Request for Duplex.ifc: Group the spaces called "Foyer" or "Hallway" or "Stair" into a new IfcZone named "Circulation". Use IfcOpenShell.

First a look at what the model holds.

```python
import ifcopenshell

model = ifcopenshell.open("Duplex.ifc")
print(model.schema)
seen = {}
for space in model.by_type("IfcSpace"):
    seen[space.LongName] = seen.get(space.LongName, 0) + 1
for name, count in sorted(seen.items(), key=str):
    print(count, "x", name)
print("zones:", [z.Name for z in model.by_type("IfcZone")][:20])
```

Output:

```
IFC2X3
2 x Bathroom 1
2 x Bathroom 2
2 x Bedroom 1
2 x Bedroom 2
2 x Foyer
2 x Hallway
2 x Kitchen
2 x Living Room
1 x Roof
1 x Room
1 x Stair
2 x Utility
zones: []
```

```python
import ifcopenshell
import ifcopenshell.api.group
import ifcopenshell.api.root

model = ifcopenshell.open("Duplex.ifc")

names = {"Foyer", "Hallway", "Stair"}
spaces = [s for s in model.by_type("IfcSpace") if s.LongName in names]

zone = ifcopenshell.api.root.create_entity(model, ifc_class="IfcZone", name="Circulation")
ifcopenshell.api.group.assign_group(model, products=spaces, group=zone)
print(len(spaces), "spaces in", zone.Name)

model.write("Duplex_updated.ifc")
```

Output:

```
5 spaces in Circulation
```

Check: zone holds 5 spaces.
